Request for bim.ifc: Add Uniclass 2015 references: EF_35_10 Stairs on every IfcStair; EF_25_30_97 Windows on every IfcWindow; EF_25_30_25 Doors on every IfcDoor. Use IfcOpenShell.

First a look at what the model holds.

```python
import ifcopenshell

model = ifcopenshell.open("bim.ifc")
print(model.schema)
print("classifications:", [c.Name for c in model.by_type("IfcClassification")])
for ifc_class in ("IfcDoor", "IfcRoof", "IfcStair", "IfcWall", "IfcWindow"):
    print(ifc_class, len(model.by_type(ifc_class)))
```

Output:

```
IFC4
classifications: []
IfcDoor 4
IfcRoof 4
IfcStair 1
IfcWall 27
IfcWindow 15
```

```python
import ifcopenshell
import ifcopenshell.api.classification

model = ifcopenshell.open("bim.ifc")

system = ifcopenshell.api.classification.add_classification(model, classification="Uniclass 2015")

codes = {
    "IfcStair": ("EF_35_10", "Stairs"),
    "IfcWindow": ("EF_25_30_97", "Windows"),
    "IfcDoor": ("EF_25_30_25", "Doors"),
}
for ifc_class, (code, name) in codes.items():
    products = model.by_type(ifc_class)
    ifcopenshell.api.classification.add_reference(
        model, products=products, classification=system, identification=code, name=name
    )
    print(code, len(products))

model.write("bim_v2.ifc")
```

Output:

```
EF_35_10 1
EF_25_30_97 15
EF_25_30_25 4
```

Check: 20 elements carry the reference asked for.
